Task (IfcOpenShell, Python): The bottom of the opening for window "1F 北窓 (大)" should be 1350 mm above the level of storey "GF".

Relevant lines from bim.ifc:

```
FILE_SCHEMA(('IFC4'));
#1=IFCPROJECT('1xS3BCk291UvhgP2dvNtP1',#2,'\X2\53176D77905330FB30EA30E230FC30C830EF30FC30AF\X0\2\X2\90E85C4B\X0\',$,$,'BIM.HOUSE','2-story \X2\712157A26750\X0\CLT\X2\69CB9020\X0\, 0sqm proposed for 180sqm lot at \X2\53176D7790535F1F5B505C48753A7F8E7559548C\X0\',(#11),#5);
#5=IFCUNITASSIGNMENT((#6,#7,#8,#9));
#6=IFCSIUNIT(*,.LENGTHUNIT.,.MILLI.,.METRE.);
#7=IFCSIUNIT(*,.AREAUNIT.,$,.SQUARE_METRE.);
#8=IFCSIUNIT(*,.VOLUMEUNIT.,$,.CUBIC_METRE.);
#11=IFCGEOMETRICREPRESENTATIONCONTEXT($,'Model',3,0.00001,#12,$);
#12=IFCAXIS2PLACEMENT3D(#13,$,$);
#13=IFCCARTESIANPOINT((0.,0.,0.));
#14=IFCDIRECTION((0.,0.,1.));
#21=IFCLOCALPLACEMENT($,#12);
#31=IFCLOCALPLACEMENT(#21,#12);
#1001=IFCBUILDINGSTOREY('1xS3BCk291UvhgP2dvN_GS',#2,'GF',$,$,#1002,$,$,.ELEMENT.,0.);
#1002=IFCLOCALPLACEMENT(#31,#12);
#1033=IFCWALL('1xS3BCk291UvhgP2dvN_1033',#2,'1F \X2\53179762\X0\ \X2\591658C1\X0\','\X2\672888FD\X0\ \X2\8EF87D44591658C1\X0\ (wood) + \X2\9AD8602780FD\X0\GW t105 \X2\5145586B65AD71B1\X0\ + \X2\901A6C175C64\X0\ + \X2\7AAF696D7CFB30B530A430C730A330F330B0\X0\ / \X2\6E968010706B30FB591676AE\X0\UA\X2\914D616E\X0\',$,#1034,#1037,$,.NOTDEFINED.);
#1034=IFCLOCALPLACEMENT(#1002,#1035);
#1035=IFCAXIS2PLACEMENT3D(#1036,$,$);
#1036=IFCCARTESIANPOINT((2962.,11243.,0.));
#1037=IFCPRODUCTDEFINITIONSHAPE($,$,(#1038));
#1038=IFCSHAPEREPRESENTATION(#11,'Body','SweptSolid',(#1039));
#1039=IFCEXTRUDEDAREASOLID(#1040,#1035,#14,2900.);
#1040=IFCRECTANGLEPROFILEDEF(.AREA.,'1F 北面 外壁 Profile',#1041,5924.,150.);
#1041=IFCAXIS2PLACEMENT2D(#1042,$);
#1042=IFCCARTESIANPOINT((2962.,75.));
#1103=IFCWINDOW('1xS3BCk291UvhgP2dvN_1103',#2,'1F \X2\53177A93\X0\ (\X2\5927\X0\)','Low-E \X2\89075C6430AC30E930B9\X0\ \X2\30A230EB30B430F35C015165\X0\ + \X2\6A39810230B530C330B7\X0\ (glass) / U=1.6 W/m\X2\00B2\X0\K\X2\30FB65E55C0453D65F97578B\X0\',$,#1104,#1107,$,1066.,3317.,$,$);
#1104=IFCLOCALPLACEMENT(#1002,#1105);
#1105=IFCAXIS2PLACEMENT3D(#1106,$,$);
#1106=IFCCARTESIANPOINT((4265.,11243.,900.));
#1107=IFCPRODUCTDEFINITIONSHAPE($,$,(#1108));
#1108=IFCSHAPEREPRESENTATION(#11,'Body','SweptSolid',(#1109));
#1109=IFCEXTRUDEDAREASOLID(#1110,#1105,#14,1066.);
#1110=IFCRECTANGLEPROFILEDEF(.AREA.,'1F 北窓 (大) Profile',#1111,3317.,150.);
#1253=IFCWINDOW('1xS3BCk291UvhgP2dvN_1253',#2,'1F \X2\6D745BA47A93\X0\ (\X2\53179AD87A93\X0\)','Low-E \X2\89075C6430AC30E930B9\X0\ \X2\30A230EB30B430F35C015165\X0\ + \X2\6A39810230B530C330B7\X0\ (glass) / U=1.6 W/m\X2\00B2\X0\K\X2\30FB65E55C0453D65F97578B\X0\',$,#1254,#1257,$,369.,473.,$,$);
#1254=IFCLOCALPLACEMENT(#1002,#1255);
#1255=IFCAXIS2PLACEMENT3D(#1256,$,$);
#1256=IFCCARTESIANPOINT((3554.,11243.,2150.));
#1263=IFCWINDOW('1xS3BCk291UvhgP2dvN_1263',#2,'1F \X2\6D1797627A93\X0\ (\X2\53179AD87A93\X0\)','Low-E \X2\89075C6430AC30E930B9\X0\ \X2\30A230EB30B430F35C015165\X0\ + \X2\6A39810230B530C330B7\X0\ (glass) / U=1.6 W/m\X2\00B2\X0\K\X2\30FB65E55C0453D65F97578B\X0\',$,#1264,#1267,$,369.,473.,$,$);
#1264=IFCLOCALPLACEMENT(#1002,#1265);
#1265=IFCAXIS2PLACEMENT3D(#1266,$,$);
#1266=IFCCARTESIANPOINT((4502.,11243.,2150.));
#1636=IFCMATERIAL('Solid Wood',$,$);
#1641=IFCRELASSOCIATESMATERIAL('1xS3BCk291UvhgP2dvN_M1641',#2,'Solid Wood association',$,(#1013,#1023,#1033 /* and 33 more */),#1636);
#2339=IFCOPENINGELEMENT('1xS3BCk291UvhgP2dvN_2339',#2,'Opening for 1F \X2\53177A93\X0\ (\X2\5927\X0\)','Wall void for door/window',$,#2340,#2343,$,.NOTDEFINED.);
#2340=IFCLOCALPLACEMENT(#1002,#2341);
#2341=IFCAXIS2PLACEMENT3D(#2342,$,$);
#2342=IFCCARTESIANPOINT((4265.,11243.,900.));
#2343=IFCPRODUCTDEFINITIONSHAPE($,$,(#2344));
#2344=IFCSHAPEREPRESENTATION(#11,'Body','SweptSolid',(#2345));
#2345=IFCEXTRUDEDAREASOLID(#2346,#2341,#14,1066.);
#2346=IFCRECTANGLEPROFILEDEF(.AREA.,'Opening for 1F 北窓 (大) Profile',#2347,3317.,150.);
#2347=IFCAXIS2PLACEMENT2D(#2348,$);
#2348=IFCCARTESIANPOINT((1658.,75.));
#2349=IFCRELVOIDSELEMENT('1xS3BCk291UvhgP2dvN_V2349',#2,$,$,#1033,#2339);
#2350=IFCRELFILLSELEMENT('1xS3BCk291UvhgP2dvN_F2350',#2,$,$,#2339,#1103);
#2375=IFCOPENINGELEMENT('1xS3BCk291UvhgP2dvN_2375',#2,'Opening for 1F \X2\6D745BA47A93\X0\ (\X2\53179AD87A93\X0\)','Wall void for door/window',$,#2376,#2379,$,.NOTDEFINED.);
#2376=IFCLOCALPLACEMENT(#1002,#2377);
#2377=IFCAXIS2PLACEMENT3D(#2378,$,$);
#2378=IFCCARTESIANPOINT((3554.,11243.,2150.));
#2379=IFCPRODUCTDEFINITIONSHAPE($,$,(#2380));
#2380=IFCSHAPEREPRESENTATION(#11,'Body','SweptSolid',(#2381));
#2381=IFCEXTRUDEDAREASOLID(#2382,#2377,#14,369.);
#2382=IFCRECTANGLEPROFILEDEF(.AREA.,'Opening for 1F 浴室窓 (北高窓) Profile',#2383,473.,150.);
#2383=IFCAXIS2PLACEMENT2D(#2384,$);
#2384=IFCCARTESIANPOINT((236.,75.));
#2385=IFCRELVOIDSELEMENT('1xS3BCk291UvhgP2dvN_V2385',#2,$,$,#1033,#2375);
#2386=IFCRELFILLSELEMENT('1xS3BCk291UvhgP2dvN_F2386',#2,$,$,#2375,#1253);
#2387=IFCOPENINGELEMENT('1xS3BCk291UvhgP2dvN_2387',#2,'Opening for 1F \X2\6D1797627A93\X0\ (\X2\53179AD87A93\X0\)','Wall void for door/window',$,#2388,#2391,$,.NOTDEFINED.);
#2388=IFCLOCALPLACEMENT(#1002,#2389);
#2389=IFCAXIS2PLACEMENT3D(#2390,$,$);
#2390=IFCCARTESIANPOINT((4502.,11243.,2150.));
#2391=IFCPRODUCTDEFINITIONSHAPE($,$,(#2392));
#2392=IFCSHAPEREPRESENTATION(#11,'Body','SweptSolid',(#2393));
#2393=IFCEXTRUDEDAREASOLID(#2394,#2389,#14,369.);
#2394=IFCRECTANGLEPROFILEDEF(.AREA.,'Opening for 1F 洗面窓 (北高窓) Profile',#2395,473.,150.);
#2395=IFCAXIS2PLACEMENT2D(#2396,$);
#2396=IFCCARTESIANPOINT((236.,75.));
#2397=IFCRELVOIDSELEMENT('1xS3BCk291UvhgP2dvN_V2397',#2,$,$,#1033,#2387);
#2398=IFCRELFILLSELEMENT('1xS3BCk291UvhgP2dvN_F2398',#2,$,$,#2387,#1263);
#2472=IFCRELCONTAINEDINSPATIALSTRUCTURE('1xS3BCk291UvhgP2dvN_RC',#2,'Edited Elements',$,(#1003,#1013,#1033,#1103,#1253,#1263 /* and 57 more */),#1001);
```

```python
import numpy as np
import ifcopenshell
import ifcopenshell.api.geometry
import ifcopenshell.geom
import ifcopenshell.util.element
import ifcopenshell.util.placement
import ifcopenshell.util.shape
import ifcopenshell.util.unit

model = ifcopenshell.open("bim.ifc")
unit_scale = ifcopenshell.util.unit.calculate_unit_scale(model)

window = model.by_guid("1xS3BCk291UvhgP2dvN_1103")
opening = window.FillsVoids[0].RelatingOpeningElement
storey = ifcopenshell.util.element.get_container(window, ifc_class="IfcBuildingStorey")
level = ifcopenshell.util.placement.get_local_placement(storey.ObjectPlacement)[2, 3]

# The opening's origin need not be at the sill, so measure its lowest point.
shape = ifcopenshell.geom.create_shape(ifcopenshell.geom.settings(), opening)
bottom = ifcopenshell.util.shape.get_shape_bottom_elevation(shape, shape.geometry) / unit_scale
dz = level + 1350.0 - bottom

shift = np.array([0.0, 0.0, dz])
# The window is not placed relative to its opening, so move both.
for product in (opening, window):
    matrix = ifcopenshell.util.placement.get_local_placement(product.ObjectPlacement)
    matrix[:3, 3] += shift
    ifcopenshell.api.geometry.edit_object_placement(model, product=product, matrix=matrix, is_si=False)

print(f"moved by {dz * unit_scale:+.3f} m")

model.write("bim_updated.ifc")
```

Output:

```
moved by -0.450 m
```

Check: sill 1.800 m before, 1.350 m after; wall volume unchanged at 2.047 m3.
